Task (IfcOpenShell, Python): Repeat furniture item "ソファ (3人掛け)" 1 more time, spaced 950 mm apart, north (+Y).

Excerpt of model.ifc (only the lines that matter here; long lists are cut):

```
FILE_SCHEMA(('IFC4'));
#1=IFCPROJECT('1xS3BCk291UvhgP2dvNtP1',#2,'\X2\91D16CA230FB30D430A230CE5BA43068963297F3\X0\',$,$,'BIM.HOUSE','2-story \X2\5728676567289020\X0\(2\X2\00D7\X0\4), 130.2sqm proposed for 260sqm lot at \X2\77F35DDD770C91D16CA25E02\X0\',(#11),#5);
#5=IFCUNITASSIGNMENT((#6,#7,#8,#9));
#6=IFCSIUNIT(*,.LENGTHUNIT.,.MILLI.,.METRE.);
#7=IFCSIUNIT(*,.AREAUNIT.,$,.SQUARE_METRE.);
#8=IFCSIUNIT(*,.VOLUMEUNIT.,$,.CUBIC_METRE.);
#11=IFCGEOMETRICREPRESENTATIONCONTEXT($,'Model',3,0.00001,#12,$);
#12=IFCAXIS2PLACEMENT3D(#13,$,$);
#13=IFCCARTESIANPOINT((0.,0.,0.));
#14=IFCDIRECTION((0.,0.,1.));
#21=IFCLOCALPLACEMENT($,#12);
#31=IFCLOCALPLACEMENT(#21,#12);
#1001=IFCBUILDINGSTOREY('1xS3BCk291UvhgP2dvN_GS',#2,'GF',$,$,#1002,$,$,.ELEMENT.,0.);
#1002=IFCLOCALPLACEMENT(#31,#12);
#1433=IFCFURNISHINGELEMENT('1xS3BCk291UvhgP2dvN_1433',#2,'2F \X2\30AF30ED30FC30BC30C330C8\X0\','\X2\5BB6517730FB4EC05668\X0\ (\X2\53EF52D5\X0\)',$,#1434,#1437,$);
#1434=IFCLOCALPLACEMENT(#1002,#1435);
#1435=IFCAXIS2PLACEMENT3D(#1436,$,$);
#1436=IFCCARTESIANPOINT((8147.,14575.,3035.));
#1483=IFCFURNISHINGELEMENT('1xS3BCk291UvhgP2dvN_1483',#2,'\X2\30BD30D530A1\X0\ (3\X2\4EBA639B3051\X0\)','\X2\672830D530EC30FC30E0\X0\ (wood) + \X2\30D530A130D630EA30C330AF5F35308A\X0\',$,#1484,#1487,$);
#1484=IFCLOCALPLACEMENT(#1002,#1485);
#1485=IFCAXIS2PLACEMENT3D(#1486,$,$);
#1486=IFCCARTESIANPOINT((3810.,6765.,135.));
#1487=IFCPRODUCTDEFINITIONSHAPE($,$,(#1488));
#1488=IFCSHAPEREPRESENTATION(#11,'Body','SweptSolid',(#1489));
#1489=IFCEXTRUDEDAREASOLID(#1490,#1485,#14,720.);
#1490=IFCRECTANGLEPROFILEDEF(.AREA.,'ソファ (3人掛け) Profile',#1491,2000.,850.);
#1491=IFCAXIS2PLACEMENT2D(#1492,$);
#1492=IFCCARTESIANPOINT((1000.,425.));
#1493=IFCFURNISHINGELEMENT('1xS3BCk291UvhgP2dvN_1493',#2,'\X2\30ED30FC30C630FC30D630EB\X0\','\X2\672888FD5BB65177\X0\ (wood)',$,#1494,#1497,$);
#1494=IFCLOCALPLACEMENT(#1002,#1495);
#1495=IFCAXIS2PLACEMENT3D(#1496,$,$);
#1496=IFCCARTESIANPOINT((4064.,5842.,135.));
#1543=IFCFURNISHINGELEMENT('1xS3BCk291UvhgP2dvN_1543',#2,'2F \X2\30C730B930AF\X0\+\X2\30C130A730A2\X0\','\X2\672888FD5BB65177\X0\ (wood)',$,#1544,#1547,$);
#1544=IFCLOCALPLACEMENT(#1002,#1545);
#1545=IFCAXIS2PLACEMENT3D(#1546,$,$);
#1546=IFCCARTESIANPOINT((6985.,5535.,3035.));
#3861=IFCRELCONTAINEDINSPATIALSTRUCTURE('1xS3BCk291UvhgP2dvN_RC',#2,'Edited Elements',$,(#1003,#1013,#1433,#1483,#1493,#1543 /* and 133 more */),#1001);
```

```python
import numpy as np
import ifcopenshell
import ifcopenshell.api.geometry
import ifcopenshell.api.root
import ifcopenshell.util.element
import ifcopenshell.util.placement

model = ifcopenshell.open("model.ifc")


def reuse_history(source, copy):
    """copy_class also copies each property set's owner history, people and application; keep the originals."""
    for rel in copy.IsDefinedBy:
        if rel.is_a("IfcRelDefinesByProperties") and (history := rel.RelatingPropertyDefinition.OwnerHistory):
            rel.RelatingPropertyDefinition.OwnerHistory = source.OwnerHistory
            ifcopenshell.util.element.remove_deep2(model, history)


source = model.by_guid("1xS3BCk291UvhgP2dvN_1483")
base = ifcopenshell.util.placement.get_local_placement(source.ObjectPlacement)
step = np.array([0.0, 1.0, 0.0]) * 950.0

for i in range(1, 2):
    copy = ifcopenshell.api.root.copy_class(model, product=source)
    copy.Representation = ifcopenshell.util.element.copy_deep(
        model, source.Representation, exclude=["IfcGeometricRepresentationContext", "IfcRepresentationMap"]
    )
    reuse_history(source, copy)
    matrix = base.copy()
    matrix[:3, 3] += i * step
    print("added at", matrix[:3, 3].round(3) + 0.0)
    ifcopenshell.api.geometry.edit_object_placement(model, product=copy, matrix=matrix, is_si=False)

model.write("model_rev.ifc")
```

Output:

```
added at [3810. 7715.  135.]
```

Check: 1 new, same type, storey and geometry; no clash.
